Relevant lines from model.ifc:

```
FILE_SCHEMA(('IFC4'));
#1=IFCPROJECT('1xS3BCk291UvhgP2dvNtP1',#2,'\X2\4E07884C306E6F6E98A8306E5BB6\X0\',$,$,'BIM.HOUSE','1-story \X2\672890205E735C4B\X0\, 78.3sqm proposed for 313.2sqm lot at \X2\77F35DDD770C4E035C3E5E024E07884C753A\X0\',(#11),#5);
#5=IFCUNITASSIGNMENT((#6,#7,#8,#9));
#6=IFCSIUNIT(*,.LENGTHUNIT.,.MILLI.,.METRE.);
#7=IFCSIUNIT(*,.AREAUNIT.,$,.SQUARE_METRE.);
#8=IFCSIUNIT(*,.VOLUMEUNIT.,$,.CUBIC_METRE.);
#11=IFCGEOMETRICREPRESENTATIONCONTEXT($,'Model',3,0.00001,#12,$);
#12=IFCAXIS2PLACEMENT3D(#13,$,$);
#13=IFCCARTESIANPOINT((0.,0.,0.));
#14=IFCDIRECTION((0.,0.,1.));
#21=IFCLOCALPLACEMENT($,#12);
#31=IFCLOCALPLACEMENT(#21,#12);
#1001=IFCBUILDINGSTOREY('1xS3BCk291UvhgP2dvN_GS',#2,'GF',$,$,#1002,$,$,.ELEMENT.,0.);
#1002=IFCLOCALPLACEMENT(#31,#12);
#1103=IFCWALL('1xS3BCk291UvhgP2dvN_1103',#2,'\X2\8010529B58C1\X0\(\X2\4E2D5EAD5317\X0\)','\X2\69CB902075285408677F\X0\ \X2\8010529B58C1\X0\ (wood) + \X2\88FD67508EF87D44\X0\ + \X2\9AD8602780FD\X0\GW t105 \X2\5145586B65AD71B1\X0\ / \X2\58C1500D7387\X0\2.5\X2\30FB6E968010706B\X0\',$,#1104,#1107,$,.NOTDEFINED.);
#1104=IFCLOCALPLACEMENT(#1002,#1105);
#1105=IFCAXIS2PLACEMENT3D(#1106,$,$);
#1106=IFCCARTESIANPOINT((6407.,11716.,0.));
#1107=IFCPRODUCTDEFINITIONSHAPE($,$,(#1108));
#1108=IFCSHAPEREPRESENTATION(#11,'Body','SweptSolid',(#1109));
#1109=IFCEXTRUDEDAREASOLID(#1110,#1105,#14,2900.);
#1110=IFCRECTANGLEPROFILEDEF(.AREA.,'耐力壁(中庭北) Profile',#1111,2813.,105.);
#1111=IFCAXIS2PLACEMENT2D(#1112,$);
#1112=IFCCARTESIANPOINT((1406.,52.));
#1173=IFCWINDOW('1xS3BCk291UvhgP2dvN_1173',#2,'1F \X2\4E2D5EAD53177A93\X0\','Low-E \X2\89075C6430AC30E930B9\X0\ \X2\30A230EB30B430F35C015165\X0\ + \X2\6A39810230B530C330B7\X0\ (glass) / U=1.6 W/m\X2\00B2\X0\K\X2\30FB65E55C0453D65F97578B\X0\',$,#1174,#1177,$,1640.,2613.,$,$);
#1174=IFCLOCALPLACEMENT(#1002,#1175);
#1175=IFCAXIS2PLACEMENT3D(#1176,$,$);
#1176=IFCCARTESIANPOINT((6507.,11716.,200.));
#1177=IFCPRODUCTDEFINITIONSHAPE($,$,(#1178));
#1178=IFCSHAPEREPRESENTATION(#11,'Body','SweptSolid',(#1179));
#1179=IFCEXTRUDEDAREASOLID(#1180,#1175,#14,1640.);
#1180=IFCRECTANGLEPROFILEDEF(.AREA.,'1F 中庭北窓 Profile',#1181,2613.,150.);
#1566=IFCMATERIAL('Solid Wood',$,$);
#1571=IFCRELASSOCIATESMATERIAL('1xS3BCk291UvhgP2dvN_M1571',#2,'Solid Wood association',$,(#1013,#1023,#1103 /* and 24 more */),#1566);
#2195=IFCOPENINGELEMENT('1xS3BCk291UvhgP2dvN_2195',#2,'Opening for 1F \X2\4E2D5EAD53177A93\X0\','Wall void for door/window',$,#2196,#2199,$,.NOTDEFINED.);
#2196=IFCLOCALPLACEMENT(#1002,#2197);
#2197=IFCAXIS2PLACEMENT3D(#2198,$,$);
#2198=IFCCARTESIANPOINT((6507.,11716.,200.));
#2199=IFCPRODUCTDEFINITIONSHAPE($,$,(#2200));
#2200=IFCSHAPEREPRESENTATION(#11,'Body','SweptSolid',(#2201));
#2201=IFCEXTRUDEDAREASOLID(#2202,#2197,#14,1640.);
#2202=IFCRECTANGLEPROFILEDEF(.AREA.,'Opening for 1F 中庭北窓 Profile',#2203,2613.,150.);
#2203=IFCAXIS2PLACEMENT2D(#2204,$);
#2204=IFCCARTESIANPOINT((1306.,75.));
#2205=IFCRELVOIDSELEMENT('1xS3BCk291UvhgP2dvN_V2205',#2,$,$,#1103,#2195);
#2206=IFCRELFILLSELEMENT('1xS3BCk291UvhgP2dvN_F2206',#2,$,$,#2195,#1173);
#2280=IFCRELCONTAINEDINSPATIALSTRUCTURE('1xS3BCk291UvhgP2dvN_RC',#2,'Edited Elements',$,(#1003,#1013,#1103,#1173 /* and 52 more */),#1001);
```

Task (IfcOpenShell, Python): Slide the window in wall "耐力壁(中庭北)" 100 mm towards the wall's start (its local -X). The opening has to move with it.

```python
import ifcopenshell
import ifcopenshell.api.geometry
import ifcopenshell.util.placement
import ifcopenshell.util.unit

model = ifcopenshell.open("model.ifc")
unit_scale = ifcopenshell.util.unit.calculate_unit_scale(model)

window = model.by_guid("1xS3BCk291UvhgP2dvN_1173")
opening = window.FillsVoids[0].RelatingOpeningElement
wall = opening.VoidsElements[0].RelatingBuildingElement

wall_matrix = ifcopenshell.util.placement.get_local_placement(wall.ObjectPlacement)
shift = wall_matrix[:3, 0] * -0.1 / unit_scale
before = ifcopenshell.util.placement.get_local_placement(window.ObjectPlacement)[:3, 3].copy()

# The window is not placed relative to its opening, so move both.
for product in (opening, window):
    matrix = ifcopenshell.util.placement.get_local_placement(product.ObjectPlacement)
    matrix[:3, 3] += shift
    ifcopenshell.api.geometry.edit_object_placement(model, product=product, matrix=matrix, is_si=False)

after = ifcopenshell.util.placement.get_local_placement(window.ObjectPlacement)[:3, 3]
print("window moved by", (after - before).round(3) + 0.0)

model.write("model_edited.ifc")
```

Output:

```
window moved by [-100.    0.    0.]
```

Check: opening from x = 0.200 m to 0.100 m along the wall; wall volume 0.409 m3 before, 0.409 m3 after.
